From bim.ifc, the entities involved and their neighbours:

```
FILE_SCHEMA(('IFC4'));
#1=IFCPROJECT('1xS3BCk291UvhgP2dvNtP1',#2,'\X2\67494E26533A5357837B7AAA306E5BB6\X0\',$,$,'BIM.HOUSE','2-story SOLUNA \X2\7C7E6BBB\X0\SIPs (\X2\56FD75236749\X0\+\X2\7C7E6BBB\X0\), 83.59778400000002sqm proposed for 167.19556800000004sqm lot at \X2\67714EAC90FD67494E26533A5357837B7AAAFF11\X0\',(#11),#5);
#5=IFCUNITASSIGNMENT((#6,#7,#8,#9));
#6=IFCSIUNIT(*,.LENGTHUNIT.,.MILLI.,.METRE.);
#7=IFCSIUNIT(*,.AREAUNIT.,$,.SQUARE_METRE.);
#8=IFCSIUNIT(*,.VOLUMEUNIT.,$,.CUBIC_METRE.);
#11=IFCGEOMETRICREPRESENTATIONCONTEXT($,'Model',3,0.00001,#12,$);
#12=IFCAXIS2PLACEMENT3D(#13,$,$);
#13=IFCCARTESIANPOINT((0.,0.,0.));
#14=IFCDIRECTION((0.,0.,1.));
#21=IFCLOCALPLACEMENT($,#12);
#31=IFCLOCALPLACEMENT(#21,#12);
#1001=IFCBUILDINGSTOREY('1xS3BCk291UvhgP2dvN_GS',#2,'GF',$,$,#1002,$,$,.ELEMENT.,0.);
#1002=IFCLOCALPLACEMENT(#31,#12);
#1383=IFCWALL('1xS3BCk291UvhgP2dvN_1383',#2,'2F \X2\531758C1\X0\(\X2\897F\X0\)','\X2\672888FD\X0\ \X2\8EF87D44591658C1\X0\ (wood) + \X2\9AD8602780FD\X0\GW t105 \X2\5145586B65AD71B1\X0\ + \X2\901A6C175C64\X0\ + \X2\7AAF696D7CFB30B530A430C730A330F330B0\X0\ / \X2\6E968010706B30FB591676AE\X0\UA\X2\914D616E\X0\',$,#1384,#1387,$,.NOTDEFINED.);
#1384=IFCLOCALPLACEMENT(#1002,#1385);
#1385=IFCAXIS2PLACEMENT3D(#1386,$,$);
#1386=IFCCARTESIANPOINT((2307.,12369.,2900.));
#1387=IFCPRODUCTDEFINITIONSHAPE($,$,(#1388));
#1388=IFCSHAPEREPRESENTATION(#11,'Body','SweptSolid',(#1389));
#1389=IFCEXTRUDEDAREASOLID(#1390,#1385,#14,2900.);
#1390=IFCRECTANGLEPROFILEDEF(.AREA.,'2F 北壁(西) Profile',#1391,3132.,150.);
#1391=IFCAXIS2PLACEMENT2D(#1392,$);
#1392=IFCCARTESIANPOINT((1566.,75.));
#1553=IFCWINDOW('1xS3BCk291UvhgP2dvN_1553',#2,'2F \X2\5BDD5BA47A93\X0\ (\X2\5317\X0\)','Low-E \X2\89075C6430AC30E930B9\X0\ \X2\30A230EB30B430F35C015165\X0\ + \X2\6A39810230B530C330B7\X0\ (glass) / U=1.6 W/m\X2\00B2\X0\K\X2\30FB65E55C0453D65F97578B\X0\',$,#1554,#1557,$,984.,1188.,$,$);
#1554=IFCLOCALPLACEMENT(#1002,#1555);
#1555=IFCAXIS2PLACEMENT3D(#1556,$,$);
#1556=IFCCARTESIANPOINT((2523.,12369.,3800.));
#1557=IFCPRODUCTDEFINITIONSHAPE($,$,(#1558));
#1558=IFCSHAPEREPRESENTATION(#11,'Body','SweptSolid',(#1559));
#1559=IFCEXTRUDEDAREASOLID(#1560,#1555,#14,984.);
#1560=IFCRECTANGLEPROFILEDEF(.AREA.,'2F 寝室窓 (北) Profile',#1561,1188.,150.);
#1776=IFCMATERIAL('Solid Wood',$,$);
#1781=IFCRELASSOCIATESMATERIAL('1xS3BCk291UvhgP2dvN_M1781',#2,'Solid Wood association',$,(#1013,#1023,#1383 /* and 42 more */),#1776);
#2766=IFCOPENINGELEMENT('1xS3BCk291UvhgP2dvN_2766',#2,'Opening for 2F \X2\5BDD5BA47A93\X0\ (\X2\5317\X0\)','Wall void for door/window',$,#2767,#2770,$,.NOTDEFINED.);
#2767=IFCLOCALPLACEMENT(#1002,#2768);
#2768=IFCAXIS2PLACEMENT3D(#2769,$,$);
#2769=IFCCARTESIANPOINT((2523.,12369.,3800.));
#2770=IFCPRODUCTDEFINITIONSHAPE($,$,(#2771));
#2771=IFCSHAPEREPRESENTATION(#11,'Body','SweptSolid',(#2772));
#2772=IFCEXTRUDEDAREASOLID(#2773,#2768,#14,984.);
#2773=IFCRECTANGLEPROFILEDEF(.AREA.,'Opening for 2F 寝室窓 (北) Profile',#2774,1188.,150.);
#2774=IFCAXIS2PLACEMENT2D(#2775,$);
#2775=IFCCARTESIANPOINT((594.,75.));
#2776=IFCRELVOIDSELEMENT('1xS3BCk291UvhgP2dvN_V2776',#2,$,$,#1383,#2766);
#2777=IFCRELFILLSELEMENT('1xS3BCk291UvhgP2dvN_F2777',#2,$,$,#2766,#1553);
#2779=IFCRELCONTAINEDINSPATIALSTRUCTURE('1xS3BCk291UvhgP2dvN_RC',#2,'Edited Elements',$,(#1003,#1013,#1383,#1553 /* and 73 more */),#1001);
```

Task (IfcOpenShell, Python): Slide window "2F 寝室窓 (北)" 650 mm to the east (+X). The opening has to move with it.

```python
import ifcopenshell
import ifcopenshell.api.geometry
import ifcopenshell.util.placement
import ifcopenshell.util.unit

model = ifcopenshell.open("bim.ifc")
unit_scale = ifcopenshell.util.unit.calculate_unit_scale(model)

window = model.by_guid("1xS3BCk291UvhgP2dvN_1553")
opening = window.FillsVoids[0].RelatingOpeningElement
wall = opening.VoidsElements[0].RelatingBuildingElement

wall_matrix = ifcopenshell.util.placement.get_local_placement(wall.ObjectPlacement)
shift = wall_matrix[:3, 0] * 0.65 / unit_scale
before = ifcopenshell.util.placement.get_local_placement(window.ObjectPlacement)[:3, 3].copy()

# The window is not placed relative to its opening, so move both.
for product in (opening, window):
    matrix = ifcopenshell.util.placement.get_local_placement(product.ObjectPlacement)
    matrix[:3, 3] += shift
    ifcopenshell.api.geometry.edit_object_placement(model, product=product, matrix=matrix, is_si=False)

after = ifcopenshell.util.placement.get_local_placement(window.ObjectPlacement)[:3, 3]
print("window moved by", (after - before).round(3) + 0.0)

model.write("bim_updated.ifc")
```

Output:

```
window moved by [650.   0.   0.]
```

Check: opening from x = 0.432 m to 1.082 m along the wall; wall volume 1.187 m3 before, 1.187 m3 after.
